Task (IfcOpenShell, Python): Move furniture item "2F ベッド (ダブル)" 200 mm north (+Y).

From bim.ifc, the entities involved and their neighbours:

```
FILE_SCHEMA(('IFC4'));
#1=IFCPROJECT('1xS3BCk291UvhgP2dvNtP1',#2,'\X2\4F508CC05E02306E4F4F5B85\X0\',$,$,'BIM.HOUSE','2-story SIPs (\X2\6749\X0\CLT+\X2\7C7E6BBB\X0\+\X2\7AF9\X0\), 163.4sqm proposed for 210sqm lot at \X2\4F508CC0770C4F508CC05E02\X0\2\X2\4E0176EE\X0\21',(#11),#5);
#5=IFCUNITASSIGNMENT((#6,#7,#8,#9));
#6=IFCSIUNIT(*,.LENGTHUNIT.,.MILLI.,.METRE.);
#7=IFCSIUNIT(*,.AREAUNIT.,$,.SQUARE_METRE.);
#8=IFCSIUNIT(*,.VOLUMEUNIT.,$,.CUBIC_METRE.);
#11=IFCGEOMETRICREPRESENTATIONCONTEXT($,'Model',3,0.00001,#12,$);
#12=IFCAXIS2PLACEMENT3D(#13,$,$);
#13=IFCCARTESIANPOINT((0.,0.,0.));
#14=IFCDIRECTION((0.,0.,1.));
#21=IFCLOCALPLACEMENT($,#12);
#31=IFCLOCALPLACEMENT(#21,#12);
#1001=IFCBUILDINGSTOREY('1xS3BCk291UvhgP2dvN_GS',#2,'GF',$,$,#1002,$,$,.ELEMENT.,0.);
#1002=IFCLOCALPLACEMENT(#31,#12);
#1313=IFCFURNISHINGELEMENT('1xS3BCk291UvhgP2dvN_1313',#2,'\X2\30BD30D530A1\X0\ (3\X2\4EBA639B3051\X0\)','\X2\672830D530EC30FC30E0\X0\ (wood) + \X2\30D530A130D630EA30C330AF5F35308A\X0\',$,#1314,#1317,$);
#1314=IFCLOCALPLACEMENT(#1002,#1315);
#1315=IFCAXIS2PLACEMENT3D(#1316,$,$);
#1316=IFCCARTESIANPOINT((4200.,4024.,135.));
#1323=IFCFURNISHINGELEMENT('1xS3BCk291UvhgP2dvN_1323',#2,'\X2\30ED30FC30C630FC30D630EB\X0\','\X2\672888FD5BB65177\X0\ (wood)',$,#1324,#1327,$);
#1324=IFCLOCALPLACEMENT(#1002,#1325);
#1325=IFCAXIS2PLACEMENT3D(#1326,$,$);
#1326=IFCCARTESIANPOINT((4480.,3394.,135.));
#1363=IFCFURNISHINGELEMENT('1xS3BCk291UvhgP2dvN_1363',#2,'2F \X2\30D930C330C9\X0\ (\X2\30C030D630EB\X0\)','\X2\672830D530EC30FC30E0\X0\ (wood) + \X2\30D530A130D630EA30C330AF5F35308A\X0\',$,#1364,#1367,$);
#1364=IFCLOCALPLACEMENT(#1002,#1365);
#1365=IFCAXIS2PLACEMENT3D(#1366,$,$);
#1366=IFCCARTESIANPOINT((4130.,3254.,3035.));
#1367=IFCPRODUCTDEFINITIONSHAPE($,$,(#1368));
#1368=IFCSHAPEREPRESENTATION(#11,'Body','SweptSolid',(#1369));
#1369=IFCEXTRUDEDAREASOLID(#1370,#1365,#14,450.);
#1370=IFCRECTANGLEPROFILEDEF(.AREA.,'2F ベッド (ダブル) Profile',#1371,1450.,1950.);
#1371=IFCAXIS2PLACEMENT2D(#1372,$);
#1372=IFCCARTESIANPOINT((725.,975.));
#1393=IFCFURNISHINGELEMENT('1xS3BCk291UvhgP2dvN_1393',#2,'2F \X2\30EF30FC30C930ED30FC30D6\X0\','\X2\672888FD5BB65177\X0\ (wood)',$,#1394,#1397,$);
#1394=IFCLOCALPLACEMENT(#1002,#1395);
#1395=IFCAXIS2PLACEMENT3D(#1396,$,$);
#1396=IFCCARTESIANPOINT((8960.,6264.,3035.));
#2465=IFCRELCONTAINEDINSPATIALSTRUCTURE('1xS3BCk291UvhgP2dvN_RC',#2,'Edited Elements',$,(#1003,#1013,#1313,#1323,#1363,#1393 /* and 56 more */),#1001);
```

```python
import ifcopenshell
import ifcopenshell.api.geometry
import ifcopenshell.util.placement

model = ifcopenshell.open("bim.ifc")

item = model.by_guid("1xS3BCk291UvhgP2dvN_1363")
matrix = ifcopenshell.util.placement.get_local_placement(item.ObjectPlacement)
matrix[1, 3] += 200.0
ifcopenshell.api.geometry.edit_object_placement(model, product=item, matrix=matrix, is_si=False)

print(ifcopenshell.util.placement.get_local_placement(item.ObjectPlacement).round(3) + 0.0)

model.write("bim-out.ifc")
```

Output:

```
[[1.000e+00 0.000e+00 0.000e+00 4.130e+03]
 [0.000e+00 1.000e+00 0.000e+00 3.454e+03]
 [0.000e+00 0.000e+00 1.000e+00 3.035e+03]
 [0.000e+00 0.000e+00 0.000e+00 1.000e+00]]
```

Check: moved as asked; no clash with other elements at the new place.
